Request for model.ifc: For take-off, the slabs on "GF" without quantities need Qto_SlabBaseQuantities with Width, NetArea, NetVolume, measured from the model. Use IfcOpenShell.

First a look at what the model holds.

```python
import ifcopenshell
import ifcopenshell.util.element
import ifcopenshell.util.unit

model = ifcopenshell.open("model.ifc")
print(model.schema)
for unit_type in ("LENGTHUNIT", "AREAUNIT", "VOLUMEUNIT"):
    print(unit_type, ifcopenshell.util.unit.calculate_unit_scale(model, unit_type))
storey = next(s for s in model.by_type("IfcBuildingStorey") if s.Name == "GF")
slabs = [e for e in ifcopenshell.util.element.get_decomposition(storey) if e.is_a("IfcSlab")]
for e in sorted(slabs, key=lambda e: e.id()):
    print(e.id(), e.is_a(), e.Name, list(ifcopenshell.util.element.get_psets(e, qtos_only=True)), sep=" | ")
```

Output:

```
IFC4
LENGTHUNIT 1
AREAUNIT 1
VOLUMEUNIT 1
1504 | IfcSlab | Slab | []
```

```python
import ifcopenshell
import ifcopenshell.api.pset
import ifcopenshell.geom
import ifcopenshell.util.element
import ifcopenshell.util.shape
import ifcopenshell.util.unit

model = ifcopenshell.open("model.ifc")
unit_scale = ifcopenshell.util.unit.calculate_unit_scale(model)
area_scale = ifcopenshell.util.unit.calculate_unit_scale(model, "AREAUNIT")
volume_scale = ifcopenshell.util.unit.calculate_unit_scale(model, "VOLUMEUNIT")
settings = ifcopenshell.geom.settings()

storey = next(s for s in model.by_type("IfcBuildingStorey") if s.Name == "GF")
slabs = [e for e in ifcopenshell.util.element.get_decomposition(storey) if e.is_a("IfcSlab")]

for e in sorted(slabs, key=lambda e: e.id()):
    if ifcopenshell.util.element.get_psets(e, qtos_only=True, should_inherit=False):
        continue
    # Geometry comes back in metres, in the element's own axes.
    shape = ifcopenshell.geom.create_shape(settings, e)
    values = {
        "Width": ifcopenshell.util.shape.get_z(shape.geometry) / unit_scale,
        "NetArea": ifcopenshell.util.shape.get_footprint_area(shape.geometry) / area_scale,
        "NetVolume": ifcopenshell.util.shape.get_volume(shape.geometry) / volume_scale,
    }
    qto = ifcopenshell.api.pset.add_qto(model, product=e, name="Qto_SlabBaseQuantities")
    ifcopenshell.api.pset.edit_qto(model, qto=qto, properties=values)
    print(e.id(), {k: round(v, 3) for k, v in values.items()})

model.write("model_rev.ifc")
```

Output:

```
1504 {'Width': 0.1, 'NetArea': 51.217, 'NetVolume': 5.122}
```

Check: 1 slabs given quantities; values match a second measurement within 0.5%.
